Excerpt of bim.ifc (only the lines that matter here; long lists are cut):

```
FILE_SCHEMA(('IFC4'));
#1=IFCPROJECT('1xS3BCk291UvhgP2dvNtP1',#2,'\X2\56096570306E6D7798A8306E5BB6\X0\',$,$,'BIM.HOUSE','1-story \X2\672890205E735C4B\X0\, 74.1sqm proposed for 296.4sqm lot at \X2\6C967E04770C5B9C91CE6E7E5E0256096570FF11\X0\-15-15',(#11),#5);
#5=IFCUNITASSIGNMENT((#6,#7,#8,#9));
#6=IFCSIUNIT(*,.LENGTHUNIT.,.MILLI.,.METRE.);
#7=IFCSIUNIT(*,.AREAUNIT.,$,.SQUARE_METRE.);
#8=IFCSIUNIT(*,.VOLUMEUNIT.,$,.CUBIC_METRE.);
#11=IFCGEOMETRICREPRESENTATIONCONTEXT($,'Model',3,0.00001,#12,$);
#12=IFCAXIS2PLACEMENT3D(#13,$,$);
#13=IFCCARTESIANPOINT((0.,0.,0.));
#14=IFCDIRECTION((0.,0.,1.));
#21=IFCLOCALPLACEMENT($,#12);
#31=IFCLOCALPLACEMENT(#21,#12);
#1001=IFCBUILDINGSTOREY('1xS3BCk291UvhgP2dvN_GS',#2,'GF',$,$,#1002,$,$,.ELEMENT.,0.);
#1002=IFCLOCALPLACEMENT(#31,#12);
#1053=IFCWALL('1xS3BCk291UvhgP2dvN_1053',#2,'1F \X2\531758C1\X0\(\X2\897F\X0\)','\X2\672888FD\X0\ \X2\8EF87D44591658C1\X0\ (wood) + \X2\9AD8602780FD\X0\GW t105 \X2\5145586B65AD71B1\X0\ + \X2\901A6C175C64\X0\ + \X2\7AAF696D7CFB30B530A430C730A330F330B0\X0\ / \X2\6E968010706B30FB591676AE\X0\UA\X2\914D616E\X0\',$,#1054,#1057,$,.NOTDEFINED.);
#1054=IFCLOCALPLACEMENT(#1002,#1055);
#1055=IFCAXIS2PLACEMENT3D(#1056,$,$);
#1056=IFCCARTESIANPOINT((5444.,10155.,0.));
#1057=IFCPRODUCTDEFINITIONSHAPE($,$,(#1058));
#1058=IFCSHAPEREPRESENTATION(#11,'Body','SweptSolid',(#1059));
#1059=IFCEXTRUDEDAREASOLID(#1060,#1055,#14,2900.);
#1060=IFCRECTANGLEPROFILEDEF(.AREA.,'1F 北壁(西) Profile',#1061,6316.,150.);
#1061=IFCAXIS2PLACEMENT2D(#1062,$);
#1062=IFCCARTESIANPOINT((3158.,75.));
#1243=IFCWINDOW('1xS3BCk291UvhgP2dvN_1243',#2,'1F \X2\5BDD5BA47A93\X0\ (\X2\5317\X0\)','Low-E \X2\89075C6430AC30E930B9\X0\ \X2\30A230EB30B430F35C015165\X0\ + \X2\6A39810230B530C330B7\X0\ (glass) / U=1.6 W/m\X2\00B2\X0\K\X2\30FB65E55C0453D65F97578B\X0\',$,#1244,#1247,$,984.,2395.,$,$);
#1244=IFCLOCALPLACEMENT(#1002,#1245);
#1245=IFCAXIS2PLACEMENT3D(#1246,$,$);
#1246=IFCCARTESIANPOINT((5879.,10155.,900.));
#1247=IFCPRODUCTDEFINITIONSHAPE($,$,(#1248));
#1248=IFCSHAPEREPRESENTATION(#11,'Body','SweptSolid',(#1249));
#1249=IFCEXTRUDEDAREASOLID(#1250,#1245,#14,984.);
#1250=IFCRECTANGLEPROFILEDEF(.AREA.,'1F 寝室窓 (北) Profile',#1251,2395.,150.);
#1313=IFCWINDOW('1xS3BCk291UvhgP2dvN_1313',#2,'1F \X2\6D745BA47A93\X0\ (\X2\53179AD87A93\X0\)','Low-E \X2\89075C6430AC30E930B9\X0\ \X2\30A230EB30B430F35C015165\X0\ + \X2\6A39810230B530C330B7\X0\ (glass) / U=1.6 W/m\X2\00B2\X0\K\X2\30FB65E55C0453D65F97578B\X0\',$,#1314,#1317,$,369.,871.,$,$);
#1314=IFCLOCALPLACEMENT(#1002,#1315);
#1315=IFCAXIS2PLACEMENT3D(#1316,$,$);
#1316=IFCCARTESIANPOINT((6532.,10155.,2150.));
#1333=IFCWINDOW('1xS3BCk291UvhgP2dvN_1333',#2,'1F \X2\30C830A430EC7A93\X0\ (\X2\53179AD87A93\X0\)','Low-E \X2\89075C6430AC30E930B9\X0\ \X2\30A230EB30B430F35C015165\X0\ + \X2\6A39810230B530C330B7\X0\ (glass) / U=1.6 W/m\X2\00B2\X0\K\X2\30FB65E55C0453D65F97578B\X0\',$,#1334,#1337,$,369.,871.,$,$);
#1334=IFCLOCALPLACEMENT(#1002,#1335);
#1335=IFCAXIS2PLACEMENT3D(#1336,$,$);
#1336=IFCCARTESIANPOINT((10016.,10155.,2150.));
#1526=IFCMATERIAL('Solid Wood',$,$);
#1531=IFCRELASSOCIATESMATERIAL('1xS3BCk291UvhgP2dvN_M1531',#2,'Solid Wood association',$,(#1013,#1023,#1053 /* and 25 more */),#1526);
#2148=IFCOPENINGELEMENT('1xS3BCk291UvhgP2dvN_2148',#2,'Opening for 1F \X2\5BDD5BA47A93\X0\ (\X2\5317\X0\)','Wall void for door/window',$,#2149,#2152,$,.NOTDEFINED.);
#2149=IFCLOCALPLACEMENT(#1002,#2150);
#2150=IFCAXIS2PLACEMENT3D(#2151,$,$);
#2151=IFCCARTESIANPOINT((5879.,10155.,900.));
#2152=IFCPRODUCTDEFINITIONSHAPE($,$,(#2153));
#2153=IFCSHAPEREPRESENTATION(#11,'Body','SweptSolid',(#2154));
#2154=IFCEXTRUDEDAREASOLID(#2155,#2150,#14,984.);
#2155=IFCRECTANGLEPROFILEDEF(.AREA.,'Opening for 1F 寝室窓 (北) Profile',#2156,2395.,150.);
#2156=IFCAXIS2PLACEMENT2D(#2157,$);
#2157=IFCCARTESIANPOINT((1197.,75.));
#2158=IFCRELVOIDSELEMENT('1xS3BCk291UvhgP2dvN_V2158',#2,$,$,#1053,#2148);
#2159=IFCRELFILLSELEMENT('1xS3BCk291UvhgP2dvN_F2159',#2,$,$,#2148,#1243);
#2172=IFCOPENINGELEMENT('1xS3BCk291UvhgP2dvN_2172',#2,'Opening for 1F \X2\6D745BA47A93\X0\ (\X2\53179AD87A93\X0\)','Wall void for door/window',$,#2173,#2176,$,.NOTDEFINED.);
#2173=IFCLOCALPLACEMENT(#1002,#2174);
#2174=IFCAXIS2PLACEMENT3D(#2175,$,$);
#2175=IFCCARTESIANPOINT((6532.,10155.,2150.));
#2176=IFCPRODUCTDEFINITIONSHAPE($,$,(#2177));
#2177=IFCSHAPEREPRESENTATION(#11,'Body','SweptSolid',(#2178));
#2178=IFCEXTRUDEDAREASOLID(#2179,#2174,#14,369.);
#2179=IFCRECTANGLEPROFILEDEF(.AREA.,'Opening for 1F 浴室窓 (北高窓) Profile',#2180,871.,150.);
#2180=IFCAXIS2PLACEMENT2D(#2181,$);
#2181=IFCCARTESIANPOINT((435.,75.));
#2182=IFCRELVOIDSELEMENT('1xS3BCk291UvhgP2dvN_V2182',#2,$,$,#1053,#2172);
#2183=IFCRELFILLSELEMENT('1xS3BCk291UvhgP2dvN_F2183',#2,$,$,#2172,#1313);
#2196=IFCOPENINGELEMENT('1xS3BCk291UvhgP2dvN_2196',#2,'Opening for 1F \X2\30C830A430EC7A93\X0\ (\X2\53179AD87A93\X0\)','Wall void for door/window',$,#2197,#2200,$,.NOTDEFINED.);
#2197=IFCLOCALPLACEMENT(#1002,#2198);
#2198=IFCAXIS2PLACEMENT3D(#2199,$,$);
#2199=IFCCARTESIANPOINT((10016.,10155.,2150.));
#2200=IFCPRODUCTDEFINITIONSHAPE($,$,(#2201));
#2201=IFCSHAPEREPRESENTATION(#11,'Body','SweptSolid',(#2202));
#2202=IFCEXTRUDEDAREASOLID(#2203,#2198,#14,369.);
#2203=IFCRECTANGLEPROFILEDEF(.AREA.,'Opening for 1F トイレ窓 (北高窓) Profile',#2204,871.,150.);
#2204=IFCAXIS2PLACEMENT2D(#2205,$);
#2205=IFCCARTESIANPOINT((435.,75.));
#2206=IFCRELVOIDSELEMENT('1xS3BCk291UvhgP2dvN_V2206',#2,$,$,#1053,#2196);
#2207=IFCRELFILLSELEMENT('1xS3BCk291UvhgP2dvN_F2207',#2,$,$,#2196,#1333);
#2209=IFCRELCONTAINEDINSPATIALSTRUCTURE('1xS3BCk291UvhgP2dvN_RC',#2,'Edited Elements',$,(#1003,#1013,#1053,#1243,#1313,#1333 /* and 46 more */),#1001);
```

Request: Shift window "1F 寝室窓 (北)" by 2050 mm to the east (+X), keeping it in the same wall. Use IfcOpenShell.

```python
import ifcopenshell
import ifcopenshell.api.geometry
import ifcopenshell.util.placement
import ifcopenshell.util.unit

model = ifcopenshell.open("bim.ifc")
unit_scale = ifcopenshell.util.unit.calculate_unit_scale(model)

window = model.by_guid("1xS3BCk291UvhgP2dvN_1243")
opening = window.FillsVoids[0].RelatingOpeningElement
wall = opening.VoidsElements[0].RelatingBuildingElement

wall_matrix = ifcopenshell.util.placement.get_local_placement(wall.ObjectPlacement)
shift = wall_matrix[:3, 0] * 2.05 / unit_scale
before = ifcopenshell.util.placement.get_local_placement(window.ObjectPlacement)[:3, 3].copy()

# The window is not placed relative to its opening, so move both.
for product in (opening, window):
    matrix = ifcopenshell.util.placement.get_local_placement(product.ObjectPlacement)
    matrix[:3, 3] += shift
    ifcopenshell.api.geometry.edit_object_placement(model, product=product, matrix=matrix, is_si=False)

after = ifcopenshell.util.placement.get_local_placement(window.ObjectPlacement)[:3, 3]
print("window moved by", (after - before).round(3) + 0.0)

model.write("bim_updated.ifc")
```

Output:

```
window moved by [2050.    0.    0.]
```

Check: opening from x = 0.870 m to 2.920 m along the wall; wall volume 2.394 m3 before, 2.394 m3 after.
